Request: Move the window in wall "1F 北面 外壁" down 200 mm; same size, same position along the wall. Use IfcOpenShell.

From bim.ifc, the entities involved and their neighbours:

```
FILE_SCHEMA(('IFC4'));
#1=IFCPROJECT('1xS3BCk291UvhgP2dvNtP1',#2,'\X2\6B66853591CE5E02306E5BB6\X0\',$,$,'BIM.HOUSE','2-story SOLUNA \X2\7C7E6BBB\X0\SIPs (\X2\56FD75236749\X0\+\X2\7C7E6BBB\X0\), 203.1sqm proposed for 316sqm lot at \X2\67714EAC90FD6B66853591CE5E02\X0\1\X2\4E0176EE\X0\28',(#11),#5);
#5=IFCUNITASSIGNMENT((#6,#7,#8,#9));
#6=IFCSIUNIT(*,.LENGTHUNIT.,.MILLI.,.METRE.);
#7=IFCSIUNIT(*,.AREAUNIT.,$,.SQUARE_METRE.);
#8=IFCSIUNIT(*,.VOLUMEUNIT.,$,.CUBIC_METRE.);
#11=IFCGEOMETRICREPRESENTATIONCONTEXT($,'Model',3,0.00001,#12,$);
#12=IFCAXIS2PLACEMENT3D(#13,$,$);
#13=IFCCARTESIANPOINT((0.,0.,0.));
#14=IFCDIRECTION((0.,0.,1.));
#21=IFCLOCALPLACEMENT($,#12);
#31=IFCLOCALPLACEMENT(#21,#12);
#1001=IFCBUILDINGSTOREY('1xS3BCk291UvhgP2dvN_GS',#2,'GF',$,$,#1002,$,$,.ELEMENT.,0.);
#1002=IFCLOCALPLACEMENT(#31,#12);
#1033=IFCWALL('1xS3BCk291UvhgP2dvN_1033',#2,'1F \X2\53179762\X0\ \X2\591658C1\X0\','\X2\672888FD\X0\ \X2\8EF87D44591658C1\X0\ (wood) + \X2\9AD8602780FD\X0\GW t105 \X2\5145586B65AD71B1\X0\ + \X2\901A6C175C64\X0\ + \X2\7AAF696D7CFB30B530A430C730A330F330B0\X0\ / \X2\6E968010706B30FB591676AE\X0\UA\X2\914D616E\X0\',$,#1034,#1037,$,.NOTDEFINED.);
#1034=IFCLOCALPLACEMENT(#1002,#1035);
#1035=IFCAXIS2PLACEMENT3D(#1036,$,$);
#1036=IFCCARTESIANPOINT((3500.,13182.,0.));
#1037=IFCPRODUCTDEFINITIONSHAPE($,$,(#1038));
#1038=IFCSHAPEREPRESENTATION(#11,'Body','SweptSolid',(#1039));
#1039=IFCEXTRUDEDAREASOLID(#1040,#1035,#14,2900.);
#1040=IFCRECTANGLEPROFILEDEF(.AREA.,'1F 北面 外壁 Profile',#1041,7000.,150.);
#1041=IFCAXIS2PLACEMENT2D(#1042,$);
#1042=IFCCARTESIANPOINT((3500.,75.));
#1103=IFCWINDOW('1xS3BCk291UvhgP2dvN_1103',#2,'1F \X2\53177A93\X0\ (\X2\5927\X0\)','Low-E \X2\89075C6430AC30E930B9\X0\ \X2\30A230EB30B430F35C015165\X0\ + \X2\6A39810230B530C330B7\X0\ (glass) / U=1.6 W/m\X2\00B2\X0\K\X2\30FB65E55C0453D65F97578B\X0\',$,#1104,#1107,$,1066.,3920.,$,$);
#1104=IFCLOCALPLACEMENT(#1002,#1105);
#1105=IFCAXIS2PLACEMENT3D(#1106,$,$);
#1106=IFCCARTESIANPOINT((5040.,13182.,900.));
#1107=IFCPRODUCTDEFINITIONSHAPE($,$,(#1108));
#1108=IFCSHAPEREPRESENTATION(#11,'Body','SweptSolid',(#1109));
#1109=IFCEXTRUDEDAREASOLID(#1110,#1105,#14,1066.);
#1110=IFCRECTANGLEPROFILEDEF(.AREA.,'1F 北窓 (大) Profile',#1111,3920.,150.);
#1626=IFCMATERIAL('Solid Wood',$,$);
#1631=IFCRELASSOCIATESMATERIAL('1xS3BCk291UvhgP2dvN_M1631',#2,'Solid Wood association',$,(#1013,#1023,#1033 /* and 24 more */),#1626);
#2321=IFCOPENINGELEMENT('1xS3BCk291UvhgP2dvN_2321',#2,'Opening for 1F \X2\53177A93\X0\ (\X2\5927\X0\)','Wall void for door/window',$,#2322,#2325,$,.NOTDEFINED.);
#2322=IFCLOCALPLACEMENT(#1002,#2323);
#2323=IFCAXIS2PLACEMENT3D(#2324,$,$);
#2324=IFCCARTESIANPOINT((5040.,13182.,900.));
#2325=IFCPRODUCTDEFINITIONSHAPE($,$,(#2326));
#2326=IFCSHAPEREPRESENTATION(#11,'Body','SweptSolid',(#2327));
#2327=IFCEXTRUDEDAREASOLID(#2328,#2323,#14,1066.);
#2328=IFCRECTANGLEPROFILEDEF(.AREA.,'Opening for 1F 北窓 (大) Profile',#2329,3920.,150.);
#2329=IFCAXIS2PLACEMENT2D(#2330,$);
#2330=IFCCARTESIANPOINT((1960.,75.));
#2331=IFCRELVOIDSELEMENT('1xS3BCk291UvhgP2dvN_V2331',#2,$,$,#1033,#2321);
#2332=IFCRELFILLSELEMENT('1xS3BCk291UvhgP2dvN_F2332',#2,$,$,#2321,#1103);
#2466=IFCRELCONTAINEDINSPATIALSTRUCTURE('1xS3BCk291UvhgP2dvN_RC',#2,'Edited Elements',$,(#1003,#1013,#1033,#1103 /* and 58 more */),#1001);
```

```python
import numpy as np
import ifcopenshell
import ifcopenshell.api.geometry
import ifcopenshell.util.placement
import ifcopenshell.util.unit

model = ifcopenshell.open("bim.ifc")
unit_scale = ifcopenshell.util.unit.calculate_unit_scale(model)

window = model.by_guid("1xS3BCk291UvhgP2dvN_1103")
opening = window.FillsVoids[0].RelatingOpeningElement
dz = -200.0

shift = np.array([0.0, 0.0, dz])
# The window is not placed relative to its opening, so move both.
for product in (opening, window):
    matrix = ifcopenshell.util.placement.get_local_placement(product.ObjectPlacement)
    matrix[:3, 3] += shift
    ifcopenshell.api.geometry.edit_object_placement(model, product=product, matrix=matrix, is_si=False)

print(f"moved by {dz * unit_scale:+.3f} m")

model.write("bim_v2.ifc")
```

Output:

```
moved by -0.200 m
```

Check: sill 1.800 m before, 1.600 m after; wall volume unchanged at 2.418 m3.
